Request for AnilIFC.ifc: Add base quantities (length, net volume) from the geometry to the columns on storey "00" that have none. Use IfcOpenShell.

First a look at what the model holds.

```python
import ifcopenshell
import ifcopenshell.util.element
import ifcopenshell.util.unit

model = ifcopenshell.open("AnilIFC.ifc")
print(model.schema)
for unit_type in ("LENGTHUNIT", "AREAUNIT", "VOLUMEUNIT"):
    print(unit_type, ifcopenshell.util.unit.calculate_unit_scale(model, unit_type))
storey = next(s for s in model.by_type("IfcBuildingStorey") if s.Name == "00")
columns = [e for e in ifcopenshell.util.element.get_decomposition(storey) if e.is_a("IfcColumn")]
for e in sorted(columns, key=lambda e: e.id()):
    print(e.id(), e.is_a(), e.Name, list(ifcopenshell.util.element.get_psets(e, qtos_only=True)), sep=" | ")
```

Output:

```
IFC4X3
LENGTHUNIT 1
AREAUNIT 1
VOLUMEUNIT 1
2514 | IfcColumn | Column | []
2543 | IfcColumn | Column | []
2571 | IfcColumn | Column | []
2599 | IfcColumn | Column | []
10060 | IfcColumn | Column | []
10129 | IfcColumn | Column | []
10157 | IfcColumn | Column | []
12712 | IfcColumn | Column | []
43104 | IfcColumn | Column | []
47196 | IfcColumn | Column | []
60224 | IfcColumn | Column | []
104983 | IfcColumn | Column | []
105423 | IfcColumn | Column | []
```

```python
import ifcopenshell
import ifcopenshell.api.pset
import ifcopenshell.geom
import ifcopenshell.util.element
import ifcopenshell.util.shape
import ifcopenshell.util.unit

model = ifcopenshell.open("AnilIFC.ifc")
unit_scale = ifcopenshell.util.unit.calculate_unit_scale(model)
volume_scale = ifcopenshell.util.unit.calculate_unit_scale(model, "VOLUMEUNIT")
settings = ifcopenshell.geom.settings()

storey = next(s for s in model.by_type("IfcBuildingStorey") if s.Name == "00")
columns = [e for e in ifcopenshell.util.element.get_decomposition(storey) if e.is_a("IfcColumn")]

for e in sorted(columns, key=lambda e: e.id()):
    if ifcopenshell.util.element.get_psets(e, qtos_only=True, should_inherit=False):
        continue
    # Geometry comes back in metres, in the element's own axes.
    shape = ifcopenshell.geom.create_shape(settings, e)
    values = {
        "Length": ifcopenshell.util.shape.get_z(shape.geometry) / unit_scale,
        "NetVolume": ifcopenshell.util.shape.get_volume(shape.geometry) / volume_scale,
    }
    qto = ifcopenshell.api.pset.add_qto(model, product=e, name="Qto_ColumnBaseQuantities")
    ifcopenshell.api.pset.edit_qto(model, qto=qto, properties=values)
    print(e.id(), {k: round(v, 3) for k, v in values.items()})

model.write("AnilIFC_updated.ifc")
```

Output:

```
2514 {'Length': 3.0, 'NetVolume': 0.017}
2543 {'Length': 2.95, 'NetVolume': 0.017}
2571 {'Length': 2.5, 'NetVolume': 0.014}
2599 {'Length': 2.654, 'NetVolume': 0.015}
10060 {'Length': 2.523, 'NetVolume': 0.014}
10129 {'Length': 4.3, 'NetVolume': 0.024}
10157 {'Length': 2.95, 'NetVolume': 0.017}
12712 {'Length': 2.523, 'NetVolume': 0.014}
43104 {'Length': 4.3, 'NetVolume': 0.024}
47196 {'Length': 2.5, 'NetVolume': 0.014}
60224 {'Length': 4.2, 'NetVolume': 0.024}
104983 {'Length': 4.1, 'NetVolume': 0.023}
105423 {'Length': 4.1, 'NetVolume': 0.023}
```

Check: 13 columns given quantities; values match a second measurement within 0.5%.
